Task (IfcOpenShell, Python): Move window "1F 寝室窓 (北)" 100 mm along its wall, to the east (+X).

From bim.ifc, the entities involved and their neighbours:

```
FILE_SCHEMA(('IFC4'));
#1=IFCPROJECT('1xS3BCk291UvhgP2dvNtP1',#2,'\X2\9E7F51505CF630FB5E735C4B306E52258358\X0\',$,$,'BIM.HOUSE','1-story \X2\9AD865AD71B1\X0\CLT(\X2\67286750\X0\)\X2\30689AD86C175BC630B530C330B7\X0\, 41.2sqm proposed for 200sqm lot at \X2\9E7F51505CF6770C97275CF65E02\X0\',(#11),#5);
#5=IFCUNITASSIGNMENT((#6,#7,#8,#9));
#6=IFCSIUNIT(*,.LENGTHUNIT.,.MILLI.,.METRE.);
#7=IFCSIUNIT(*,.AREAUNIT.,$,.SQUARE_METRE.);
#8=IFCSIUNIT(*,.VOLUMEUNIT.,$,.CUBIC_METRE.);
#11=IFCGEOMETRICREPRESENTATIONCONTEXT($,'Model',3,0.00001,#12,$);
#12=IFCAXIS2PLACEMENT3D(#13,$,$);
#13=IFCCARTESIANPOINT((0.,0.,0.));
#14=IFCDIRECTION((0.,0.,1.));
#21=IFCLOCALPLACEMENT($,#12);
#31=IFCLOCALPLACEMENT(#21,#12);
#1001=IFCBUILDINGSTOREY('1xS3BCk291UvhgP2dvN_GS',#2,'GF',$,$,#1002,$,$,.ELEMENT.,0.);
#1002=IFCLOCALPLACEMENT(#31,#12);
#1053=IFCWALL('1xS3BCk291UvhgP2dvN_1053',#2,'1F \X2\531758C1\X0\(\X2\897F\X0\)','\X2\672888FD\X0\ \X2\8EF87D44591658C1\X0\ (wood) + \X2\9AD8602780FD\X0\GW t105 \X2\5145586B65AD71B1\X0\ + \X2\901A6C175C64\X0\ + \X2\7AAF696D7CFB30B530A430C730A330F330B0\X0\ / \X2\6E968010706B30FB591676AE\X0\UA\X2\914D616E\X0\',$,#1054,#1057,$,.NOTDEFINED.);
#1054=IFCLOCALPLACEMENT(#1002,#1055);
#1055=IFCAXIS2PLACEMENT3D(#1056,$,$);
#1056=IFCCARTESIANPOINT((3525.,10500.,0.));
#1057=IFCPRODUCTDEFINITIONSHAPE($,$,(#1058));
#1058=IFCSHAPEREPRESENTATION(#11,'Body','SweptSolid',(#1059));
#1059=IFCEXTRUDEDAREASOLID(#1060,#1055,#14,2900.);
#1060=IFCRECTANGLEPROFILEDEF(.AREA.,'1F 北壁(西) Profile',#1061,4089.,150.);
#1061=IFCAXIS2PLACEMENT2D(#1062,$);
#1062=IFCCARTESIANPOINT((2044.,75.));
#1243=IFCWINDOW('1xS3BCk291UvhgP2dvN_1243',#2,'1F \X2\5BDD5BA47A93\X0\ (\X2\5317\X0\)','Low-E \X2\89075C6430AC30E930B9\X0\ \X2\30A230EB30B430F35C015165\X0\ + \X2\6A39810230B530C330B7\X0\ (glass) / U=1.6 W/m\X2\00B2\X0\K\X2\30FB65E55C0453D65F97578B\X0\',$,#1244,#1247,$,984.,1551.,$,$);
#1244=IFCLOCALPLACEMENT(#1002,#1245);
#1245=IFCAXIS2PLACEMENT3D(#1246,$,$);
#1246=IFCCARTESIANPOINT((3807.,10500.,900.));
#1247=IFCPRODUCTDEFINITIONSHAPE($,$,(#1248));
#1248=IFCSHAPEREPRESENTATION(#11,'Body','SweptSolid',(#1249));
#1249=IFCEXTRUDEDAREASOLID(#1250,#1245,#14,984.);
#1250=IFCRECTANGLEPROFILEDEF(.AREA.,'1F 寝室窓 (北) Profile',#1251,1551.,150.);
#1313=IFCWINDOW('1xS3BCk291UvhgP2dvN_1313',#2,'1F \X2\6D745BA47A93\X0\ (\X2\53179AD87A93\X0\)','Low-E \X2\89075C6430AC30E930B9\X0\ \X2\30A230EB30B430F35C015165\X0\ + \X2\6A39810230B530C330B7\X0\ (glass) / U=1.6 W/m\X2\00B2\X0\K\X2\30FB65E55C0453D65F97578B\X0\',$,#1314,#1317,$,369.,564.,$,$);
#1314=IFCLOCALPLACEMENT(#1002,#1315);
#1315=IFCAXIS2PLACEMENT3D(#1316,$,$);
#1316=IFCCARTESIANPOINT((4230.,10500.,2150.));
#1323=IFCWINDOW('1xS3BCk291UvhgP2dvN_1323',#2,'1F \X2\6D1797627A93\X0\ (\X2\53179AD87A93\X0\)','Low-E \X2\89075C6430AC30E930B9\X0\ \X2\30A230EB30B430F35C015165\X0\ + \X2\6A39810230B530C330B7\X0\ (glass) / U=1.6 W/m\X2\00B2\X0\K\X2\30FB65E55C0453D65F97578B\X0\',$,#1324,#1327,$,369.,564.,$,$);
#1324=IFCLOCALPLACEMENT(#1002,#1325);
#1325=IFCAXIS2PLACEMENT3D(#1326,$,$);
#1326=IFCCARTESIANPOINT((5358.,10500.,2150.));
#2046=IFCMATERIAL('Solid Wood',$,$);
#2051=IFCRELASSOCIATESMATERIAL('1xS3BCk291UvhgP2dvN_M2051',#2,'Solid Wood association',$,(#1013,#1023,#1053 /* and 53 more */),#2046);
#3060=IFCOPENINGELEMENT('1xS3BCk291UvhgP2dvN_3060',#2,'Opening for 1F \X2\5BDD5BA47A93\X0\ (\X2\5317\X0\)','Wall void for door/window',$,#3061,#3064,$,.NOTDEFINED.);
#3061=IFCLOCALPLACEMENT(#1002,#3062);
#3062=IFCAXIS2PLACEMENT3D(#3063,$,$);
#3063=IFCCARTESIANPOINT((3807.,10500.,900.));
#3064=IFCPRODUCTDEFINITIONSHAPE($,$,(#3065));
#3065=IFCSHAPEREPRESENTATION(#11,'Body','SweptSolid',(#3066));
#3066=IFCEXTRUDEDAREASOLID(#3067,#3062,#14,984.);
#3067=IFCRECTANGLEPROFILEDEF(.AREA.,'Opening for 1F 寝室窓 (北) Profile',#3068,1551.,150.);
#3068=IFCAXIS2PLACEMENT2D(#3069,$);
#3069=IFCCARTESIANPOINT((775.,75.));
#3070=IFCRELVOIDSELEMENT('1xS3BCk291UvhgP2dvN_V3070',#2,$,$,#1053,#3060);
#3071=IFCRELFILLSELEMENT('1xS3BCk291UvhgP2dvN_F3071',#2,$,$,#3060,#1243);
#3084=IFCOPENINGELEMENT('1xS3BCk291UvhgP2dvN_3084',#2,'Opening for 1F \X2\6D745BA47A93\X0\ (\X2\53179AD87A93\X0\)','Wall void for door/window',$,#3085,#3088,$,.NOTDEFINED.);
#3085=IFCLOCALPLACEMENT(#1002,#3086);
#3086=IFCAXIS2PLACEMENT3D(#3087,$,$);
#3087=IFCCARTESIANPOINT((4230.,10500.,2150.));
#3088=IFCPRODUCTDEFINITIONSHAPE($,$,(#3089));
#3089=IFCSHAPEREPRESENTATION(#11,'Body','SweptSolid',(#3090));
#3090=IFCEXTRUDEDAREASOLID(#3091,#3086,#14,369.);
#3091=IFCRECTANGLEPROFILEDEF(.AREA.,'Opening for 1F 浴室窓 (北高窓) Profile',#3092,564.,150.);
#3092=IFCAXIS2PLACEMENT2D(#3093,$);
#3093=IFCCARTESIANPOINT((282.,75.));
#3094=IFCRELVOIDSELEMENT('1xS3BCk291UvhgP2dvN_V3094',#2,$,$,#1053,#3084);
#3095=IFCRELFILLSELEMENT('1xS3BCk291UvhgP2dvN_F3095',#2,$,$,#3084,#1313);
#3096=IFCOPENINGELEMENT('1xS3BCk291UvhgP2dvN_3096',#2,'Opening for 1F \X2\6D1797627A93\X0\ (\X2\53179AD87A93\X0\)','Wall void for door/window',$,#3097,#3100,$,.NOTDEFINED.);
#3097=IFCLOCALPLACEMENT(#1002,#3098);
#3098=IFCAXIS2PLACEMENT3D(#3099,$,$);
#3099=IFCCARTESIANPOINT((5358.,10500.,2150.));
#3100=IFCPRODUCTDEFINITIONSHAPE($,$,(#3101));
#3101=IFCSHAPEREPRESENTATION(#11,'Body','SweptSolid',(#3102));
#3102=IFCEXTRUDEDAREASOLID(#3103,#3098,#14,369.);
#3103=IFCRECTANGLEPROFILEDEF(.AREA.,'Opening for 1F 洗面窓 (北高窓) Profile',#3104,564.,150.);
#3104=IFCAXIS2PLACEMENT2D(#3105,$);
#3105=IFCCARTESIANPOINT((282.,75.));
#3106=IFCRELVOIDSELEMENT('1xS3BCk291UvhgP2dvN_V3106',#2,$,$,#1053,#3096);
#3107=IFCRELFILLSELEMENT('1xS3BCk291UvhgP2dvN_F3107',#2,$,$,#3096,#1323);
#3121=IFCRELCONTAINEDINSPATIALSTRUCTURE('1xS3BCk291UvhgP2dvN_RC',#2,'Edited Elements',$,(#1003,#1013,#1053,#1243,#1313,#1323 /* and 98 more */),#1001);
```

```python
import ifcopenshell
import ifcopenshell.api.geometry
import ifcopenshell.util.placement
import ifcopenshell.util.unit

model = ifcopenshell.open("bim.ifc")
unit_scale = ifcopenshell.util.unit.calculate_unit_scale(model)

window = model.by_id(1243)
opening = window.FillsVoids[0].RelatingOpeningElement
wall = opening.VoidsElements[0].RelatingBuildingElement

wall_matrix = ifcopenshell.util.placement.get_local_placement(wall.ObjectPlacement)
shift = wall_matrix[:3, 0] * 0.1 / unit_scale
before = ifcopenshell.util.placement.get_local_placement(window.ObjectPlacement)[:3, 3].copy()

# The window is not placed relative to its opening, so move both.
for product in (opening, window):
    matrix = ifcopenshell.util.placement.get_local_placement(product.ObjectPlacement)
    matrix[:3, 3] += shift
    ifcopenshell.api.geometry.edit_object_placement(model, product=product, matrix=matrix, is_si=False)

after = ifcopenshell.util.placement.get_local_placement(window.ObjectPlacement)[:3, 3]
print("window moved by", (after - before).round(3) + 0.0)

model.write("bim_edited.ifc")
```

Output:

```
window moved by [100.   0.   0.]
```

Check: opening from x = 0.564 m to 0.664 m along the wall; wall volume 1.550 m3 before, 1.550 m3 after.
